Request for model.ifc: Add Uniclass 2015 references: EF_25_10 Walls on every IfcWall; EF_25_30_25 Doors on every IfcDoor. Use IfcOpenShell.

First a look at what the model holds.

```python
import ifcopenshell

model = ifcopenshell.open("model.ifc")
print(model.schema)
print("classifications:", [c.Name for c in model.by_type("IfcClassification")])
for ifc_class in ("IfcDoor", "IfcRoof", "IfcStair", "IfcWall", "IfcWindow"):
    print(ifc_class, len(model.by_type(ifc_class)))
```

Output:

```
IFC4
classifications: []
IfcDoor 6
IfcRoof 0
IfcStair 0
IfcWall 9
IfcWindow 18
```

```python
import ifcopenshell
import ifcopenshell.api.classification

model = ifcopenshell.open("model.ifc")

system = ifcopenshell.api.classification.add_classification(model, classification="Uniclass 2015")

codes = {
    "IfcWall": ("EF_25_10", "Walls"),
    "IfcDoor": ("EF_25_30_25", "Doors"),
}
for ifc_class, (code, name) in codes.items():
    products = model.by_type(ifc_class)
    ifcopenshell.api.classification.add_reference(
        model, products=products, classification=system, identification=code, name=name
    )
    print(code, len(products))

model.write("model_v2.ifc")
```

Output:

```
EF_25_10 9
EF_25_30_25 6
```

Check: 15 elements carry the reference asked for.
